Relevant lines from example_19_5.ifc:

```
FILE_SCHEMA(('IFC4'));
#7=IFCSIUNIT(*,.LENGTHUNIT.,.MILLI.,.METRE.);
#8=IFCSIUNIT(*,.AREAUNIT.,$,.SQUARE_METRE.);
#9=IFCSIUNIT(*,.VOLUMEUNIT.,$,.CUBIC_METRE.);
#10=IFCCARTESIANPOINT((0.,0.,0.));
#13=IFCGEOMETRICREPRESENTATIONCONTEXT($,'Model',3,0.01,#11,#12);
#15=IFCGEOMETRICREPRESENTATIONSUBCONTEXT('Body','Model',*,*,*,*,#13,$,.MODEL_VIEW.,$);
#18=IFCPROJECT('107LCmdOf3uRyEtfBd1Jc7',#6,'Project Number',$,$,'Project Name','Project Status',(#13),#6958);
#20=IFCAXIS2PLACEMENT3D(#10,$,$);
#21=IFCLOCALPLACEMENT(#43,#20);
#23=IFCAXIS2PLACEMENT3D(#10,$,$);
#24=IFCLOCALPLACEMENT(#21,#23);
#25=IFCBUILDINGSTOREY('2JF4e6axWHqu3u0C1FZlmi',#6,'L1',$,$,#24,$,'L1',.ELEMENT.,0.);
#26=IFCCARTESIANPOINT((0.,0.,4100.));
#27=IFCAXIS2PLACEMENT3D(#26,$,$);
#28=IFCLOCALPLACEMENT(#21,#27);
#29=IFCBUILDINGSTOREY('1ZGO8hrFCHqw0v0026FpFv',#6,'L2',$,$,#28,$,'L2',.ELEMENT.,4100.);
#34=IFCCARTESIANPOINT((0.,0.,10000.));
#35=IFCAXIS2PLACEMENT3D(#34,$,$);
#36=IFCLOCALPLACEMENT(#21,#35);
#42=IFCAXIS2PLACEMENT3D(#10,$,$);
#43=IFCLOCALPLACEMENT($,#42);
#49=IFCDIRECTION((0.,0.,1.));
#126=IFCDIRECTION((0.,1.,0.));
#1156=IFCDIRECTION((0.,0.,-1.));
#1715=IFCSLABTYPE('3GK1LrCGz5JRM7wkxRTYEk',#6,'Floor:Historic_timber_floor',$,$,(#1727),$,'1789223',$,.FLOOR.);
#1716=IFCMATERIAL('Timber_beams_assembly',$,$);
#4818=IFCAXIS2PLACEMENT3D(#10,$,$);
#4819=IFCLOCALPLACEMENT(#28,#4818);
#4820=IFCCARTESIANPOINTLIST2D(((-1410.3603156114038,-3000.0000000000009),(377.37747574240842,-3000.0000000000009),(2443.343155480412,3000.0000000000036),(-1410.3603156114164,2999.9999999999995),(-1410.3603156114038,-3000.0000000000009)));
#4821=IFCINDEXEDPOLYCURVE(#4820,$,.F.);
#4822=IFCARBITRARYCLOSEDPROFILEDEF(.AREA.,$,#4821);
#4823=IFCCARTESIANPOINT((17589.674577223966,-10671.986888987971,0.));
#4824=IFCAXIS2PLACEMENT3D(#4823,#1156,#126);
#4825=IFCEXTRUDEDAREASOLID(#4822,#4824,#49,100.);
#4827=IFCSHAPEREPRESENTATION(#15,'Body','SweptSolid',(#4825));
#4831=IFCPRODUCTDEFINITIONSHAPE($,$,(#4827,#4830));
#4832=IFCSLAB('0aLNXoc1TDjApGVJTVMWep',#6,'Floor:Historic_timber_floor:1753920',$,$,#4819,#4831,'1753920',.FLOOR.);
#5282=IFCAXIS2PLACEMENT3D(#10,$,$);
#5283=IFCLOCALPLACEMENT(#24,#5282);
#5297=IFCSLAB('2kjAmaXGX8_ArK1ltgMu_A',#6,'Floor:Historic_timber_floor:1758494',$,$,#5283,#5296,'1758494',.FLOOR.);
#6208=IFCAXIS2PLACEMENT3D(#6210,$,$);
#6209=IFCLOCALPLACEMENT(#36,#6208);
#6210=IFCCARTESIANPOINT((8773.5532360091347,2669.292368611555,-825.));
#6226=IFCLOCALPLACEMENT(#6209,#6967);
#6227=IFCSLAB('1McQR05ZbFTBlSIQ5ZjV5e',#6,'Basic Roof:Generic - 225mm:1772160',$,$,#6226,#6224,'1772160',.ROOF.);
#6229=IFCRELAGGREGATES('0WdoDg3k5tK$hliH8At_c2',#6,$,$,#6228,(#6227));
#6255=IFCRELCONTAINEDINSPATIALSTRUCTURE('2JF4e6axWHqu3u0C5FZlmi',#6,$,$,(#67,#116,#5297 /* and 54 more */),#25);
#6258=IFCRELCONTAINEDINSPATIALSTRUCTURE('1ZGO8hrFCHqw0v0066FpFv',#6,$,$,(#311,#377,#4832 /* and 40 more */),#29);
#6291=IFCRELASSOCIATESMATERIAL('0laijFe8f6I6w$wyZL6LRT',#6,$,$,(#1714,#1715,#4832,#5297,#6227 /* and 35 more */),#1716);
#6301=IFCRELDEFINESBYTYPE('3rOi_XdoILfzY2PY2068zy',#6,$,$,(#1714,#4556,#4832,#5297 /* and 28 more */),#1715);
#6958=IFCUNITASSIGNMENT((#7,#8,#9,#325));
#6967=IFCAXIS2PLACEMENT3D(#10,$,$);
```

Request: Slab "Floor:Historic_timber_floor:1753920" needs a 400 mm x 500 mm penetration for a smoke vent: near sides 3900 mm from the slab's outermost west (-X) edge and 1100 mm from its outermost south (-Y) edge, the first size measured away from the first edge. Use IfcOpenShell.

```python
import numpy as np
import ifcopenshell
import ifcopenshell.api.feature
import ifcopenshell.api.geometry
import ifcopenshell.api.root
import ifcopenshell.geom
import ifcopenshell.util.placement
import ifcopenshell.util.representation
import ifcopenshell.util.shape
import ifcopenshell.util.unit

model = ifcopenshell.open("example_19_5.ifc")
unit_scale = ifcopenshell.util.unit.calculate_unit_scale(model)
settings = ifcopenshell.geom.settings()


def volume(element):
    """Net volume in cubic metres, openings subtracted."""
    shape = ifcopenshell.geom.create_shape(settings, element)
    return ifcopenshell.util.shape.get_volume(shape.geometry)


slab = model.by_id(4832)
before = volume(slab)

# Extent in the slab's own axes, in metres. The edges named are its -X and -Y sides.
slab_shape = ifcopenshell.geom.create_shape(settings, slab)
vertices = ifcopenshell.util.shape.get_vertices(slab_shape.geometry)
x_min, y_min, bottom = vertices.min(axis=0)
top = vertices[:, 2].max()

opening = ifcopenshell.api.root.create_entity(model, ifc_class="IfcOpeningElement", name="Smoke vent opening", predefined_type="OPENING")
context = ifcopenshell.util.representation.get_context(model, "Model", "Body", "MODEL_VIEW")
width, depth = 0.4, 0.5
outline = [(0.0, 0.0), (width, 0.0), (width, depth), (0.0, depth), (0.0, 0.0)]
# Overshoot both faces by 50 mm so the cut is clean.
shape = ifcopenshell.api.geometry.add_slab_representation(
    model, context=context, depth=top - bottom + 0.1, polyline=outline
)
ifcopenshell.api.geometry.assign_representation(model, product=opening, representation=shape)

matrix = ifcopenshell.util.placement.get_local_placement(slab.ObjectPlacement)
matrix[:, 3] = matrix @ np.append(np.array([x_min + 3.9, y_min + 1.1, bottom - 0.05]) / unit_scale, 1.0)
ifcopenshell.api.geometry.edit_object_placement(model, product=opening, matrix=matrix, is_si=False)
ifcopenshell.api.feature.add_feature(model, feature=opening, element=slab)

after = volume(slab)

print(f"slab volume {before:.3f} -> {after:.3f} m3")

model.write("example_19_5_rev.ifc")
```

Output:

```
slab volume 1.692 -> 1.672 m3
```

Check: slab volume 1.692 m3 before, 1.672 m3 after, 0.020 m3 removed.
